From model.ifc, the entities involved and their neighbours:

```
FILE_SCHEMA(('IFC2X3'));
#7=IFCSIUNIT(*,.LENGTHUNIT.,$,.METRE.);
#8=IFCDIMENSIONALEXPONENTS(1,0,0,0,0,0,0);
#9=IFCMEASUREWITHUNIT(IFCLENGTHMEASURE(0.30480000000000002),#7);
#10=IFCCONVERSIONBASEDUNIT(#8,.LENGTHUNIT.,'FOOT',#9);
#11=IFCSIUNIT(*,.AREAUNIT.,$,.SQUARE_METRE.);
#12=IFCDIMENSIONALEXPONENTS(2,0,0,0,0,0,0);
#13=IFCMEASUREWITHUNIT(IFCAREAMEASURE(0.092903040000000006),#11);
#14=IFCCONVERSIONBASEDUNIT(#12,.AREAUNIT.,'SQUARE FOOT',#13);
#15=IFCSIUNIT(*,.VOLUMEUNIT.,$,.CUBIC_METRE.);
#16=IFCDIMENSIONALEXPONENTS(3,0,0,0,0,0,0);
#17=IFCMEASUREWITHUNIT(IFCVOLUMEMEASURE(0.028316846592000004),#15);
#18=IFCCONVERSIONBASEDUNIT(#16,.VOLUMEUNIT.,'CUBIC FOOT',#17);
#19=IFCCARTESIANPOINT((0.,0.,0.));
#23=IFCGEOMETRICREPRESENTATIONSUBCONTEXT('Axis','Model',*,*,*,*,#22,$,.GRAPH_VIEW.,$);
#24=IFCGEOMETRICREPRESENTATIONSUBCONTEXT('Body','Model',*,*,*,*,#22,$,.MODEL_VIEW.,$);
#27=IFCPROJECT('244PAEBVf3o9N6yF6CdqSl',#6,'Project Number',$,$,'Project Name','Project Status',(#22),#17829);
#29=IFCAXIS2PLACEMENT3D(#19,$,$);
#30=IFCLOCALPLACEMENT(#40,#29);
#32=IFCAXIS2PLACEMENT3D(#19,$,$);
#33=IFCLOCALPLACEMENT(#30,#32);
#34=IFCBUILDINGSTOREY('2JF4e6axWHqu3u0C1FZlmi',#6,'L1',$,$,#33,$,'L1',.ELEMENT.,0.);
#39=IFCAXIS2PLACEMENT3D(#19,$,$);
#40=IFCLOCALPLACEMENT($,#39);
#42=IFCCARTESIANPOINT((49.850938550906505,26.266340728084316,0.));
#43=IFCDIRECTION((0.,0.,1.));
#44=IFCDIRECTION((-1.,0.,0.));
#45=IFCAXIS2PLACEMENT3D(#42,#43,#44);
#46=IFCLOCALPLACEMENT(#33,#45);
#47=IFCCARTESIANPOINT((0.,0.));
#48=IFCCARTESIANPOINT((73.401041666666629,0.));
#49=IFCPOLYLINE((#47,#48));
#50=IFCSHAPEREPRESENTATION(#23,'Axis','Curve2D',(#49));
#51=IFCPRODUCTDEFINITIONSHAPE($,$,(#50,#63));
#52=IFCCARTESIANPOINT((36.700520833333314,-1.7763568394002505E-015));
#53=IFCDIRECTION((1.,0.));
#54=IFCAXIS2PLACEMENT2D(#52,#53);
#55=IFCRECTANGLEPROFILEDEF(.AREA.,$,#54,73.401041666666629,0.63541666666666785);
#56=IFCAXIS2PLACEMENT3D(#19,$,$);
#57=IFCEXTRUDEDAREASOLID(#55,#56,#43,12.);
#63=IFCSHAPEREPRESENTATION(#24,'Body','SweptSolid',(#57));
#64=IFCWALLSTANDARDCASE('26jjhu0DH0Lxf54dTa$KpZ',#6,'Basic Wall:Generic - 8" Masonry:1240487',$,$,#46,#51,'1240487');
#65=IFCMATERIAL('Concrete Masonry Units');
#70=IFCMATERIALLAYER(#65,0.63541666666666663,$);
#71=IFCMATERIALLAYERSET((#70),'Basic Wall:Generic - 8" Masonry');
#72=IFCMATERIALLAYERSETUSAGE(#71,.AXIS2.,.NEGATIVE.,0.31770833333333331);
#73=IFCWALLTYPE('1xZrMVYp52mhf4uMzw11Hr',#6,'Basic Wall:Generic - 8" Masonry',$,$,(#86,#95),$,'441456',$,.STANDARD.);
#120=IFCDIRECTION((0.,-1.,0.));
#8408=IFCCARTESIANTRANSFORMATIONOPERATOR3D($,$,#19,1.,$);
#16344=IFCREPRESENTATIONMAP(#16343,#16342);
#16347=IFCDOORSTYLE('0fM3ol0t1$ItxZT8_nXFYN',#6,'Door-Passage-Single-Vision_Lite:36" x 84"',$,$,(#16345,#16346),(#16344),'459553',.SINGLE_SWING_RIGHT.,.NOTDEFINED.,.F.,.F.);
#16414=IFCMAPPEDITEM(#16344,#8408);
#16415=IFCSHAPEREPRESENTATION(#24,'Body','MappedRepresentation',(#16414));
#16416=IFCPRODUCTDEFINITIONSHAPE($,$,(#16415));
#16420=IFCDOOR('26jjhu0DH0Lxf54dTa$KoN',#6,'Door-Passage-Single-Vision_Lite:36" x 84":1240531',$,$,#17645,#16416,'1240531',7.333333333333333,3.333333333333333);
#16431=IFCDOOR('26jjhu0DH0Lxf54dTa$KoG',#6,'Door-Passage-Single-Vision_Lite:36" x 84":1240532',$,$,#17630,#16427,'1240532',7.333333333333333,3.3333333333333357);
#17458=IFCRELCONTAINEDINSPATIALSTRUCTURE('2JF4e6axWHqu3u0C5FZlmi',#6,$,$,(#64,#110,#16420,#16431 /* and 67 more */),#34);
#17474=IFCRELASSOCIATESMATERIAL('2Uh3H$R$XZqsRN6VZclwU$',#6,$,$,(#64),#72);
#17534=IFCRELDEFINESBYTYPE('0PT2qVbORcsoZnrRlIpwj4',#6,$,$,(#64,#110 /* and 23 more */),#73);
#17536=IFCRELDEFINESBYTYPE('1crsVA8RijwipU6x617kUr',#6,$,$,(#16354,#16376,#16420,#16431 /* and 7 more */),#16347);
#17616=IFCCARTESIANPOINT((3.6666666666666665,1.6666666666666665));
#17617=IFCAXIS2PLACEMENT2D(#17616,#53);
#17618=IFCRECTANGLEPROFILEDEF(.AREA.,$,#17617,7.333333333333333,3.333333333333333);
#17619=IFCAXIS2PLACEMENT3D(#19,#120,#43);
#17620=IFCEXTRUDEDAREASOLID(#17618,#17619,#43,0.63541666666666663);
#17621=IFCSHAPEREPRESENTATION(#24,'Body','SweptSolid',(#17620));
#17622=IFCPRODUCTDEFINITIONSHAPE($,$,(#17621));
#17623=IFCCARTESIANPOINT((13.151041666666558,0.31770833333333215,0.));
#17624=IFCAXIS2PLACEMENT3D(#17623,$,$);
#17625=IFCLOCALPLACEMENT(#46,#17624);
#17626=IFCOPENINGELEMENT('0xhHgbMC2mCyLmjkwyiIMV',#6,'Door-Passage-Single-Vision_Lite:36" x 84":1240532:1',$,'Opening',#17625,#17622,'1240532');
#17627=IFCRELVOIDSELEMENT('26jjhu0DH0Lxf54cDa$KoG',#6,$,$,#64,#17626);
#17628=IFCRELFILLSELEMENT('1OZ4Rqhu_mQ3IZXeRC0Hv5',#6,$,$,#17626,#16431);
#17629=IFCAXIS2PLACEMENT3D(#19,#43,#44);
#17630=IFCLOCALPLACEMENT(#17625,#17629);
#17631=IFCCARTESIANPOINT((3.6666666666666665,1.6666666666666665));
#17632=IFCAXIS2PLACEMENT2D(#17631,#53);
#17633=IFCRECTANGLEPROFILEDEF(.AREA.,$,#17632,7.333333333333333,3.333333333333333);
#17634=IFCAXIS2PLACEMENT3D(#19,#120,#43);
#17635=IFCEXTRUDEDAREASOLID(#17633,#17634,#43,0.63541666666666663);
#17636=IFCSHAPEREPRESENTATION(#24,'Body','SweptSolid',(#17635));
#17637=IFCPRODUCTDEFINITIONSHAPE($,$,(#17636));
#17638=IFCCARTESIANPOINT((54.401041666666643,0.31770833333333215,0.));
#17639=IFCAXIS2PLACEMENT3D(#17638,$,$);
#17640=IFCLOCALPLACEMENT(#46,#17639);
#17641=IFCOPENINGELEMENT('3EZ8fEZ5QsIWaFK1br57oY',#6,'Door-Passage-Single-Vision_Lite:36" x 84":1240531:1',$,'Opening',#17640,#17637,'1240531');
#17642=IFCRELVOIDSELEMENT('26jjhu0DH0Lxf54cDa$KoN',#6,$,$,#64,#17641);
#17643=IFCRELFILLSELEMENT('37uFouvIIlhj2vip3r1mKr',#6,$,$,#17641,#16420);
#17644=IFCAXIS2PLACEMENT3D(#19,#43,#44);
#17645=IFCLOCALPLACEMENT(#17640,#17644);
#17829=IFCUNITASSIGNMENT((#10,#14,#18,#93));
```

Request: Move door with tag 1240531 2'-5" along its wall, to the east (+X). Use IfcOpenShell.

```python
import ifcopenshell
import ifcopenshell.api.geometry
import ifcopenshell.util.placement
import ifcopenshell.util.unit

model = ifcopenshell.open("model.ifc")
unit_scale = ifcopenshell.util.unit.calculate_unit_scale(model)

door = model.by_id(16420)
opening = door.FillsVoids[0].RelatingOpeningElement
wall = opening.VoidsElements[0].RelatingBuildingElement

wall_matrix = ifcopenshell.util.placement.get_local_placement(wall.ObjectPlacement)
shift = wall_matrix[:3, 0] * -29 * 0.0254 / unit_scale
before = ifcopenshell.util.placement.get_local_placement(door.ObjectPlacement)[:3, 3].copy()

# The door is placed relative to its opening, so it follows when the opening moves.
matrix = ifcopenshell.util.placement.get_local_placement(opening.ObjectPlacement)
matrix[:3, 3] += shift
ifcopenshell.api.geometry.edit_object_placement(
    model, product=opening, matrix=matrix, is_si=False, should_transform_children=True
)

after = ifcopenshell.util.placement.get_local_placement(door.ObjectPlacement)[:3, 3]
print("door moved by", (after - before).round(3) + 0.0)

model.write("model_rev.ifc")
```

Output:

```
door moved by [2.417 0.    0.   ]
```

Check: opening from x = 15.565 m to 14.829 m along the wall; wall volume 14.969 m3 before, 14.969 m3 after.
